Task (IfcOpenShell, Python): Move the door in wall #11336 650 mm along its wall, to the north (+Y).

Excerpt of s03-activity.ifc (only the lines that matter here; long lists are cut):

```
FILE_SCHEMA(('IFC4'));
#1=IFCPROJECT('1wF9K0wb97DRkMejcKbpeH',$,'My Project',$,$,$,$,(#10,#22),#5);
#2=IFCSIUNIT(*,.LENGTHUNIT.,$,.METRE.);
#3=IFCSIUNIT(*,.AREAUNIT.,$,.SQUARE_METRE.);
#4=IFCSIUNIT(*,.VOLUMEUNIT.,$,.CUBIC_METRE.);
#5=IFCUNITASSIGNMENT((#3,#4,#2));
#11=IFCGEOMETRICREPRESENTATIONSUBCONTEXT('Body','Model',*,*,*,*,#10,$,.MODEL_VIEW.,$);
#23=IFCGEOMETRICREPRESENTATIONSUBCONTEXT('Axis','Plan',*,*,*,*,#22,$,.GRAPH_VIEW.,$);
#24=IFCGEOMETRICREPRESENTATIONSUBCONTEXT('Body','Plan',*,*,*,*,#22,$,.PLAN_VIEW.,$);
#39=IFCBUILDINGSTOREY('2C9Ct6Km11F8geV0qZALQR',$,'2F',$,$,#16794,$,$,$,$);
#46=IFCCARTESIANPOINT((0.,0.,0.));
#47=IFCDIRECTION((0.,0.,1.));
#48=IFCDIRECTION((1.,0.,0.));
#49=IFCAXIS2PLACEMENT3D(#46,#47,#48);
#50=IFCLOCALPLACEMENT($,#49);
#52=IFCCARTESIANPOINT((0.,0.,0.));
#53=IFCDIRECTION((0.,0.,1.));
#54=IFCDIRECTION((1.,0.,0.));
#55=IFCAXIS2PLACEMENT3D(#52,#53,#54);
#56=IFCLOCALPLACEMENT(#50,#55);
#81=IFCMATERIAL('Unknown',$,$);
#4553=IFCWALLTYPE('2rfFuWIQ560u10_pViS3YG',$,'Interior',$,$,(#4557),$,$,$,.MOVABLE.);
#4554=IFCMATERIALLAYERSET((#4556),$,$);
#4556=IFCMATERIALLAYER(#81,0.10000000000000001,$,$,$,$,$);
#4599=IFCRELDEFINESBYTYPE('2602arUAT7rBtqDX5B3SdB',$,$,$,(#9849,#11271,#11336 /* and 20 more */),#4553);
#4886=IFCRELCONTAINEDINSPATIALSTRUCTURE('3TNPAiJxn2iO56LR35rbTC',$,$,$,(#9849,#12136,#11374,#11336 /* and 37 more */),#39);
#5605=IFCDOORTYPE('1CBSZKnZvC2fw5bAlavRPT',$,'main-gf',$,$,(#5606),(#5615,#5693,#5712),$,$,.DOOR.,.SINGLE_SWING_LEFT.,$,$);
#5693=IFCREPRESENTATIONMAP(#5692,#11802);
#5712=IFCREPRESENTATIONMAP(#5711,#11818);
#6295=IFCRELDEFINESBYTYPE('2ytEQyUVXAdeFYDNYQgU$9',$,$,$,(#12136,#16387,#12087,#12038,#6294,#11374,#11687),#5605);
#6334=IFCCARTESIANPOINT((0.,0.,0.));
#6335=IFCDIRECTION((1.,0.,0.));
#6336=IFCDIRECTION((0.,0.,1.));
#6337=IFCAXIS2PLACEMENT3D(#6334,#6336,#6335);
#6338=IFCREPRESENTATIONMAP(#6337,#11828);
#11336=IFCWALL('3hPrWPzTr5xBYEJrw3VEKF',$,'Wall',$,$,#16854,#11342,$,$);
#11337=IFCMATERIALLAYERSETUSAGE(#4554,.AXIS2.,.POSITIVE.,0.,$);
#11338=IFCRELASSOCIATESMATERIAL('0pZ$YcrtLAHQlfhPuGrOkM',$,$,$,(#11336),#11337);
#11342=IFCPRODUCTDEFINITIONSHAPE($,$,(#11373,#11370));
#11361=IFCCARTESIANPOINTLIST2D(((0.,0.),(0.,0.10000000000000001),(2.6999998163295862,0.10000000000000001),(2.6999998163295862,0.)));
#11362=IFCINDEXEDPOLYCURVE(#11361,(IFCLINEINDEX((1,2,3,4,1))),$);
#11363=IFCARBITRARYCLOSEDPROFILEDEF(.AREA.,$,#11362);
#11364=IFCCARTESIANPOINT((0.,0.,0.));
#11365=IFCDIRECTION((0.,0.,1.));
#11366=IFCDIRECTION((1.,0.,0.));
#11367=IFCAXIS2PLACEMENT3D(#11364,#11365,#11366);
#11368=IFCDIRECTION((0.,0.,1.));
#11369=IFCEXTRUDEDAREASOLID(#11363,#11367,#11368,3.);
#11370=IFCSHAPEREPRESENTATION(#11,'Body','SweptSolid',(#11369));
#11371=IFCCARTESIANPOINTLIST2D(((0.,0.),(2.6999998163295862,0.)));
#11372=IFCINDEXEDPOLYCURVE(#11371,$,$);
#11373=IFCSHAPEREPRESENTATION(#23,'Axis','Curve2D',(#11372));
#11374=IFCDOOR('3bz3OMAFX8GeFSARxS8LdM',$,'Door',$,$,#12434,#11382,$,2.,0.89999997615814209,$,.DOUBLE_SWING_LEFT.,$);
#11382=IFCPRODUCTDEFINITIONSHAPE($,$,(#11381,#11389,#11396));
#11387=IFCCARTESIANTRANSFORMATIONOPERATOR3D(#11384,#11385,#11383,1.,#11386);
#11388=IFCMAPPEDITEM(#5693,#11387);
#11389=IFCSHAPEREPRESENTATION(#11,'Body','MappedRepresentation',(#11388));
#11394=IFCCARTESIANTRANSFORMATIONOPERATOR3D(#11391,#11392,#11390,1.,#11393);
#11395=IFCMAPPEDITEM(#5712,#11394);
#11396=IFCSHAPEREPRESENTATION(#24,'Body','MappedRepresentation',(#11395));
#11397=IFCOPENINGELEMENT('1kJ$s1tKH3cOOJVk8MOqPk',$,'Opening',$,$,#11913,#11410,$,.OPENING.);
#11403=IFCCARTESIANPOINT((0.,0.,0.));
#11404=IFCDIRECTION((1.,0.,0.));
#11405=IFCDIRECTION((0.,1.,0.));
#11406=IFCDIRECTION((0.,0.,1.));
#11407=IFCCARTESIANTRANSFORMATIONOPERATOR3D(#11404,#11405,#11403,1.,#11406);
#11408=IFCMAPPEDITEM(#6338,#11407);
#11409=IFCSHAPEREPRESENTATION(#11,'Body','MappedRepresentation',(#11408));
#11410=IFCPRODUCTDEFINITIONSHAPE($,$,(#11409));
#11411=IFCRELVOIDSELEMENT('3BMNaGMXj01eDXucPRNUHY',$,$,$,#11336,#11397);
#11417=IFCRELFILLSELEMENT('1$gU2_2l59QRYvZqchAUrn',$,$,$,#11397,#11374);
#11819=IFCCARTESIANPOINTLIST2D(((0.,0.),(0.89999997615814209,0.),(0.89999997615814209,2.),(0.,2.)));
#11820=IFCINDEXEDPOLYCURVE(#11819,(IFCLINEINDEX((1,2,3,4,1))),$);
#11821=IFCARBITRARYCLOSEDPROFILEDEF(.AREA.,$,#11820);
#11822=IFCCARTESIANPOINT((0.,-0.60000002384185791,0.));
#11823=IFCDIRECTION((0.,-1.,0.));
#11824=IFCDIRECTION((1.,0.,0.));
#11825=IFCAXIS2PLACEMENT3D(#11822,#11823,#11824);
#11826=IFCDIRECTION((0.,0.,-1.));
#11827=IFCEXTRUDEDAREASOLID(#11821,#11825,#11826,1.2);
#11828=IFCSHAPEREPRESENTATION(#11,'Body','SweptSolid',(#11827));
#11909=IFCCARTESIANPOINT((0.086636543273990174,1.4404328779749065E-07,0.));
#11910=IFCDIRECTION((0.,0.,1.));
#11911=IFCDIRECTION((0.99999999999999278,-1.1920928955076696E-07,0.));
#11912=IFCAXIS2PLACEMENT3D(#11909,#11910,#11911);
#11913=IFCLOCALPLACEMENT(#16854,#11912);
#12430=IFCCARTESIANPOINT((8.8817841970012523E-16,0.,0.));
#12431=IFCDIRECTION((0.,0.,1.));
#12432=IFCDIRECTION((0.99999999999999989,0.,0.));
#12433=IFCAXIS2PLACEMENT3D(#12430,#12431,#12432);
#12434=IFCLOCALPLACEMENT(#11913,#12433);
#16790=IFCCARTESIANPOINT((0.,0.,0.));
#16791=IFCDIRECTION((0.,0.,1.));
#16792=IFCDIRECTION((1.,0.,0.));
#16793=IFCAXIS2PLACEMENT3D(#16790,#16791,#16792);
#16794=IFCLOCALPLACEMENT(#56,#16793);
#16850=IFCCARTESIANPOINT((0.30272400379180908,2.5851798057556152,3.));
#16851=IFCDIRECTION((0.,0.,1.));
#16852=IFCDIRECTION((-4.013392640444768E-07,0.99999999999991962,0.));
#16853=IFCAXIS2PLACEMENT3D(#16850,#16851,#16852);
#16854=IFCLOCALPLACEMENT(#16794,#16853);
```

```python
import ifcopenshell
import ifcopenshell.api.geometry
import ifcopenshell.util.placement
import ifcopenshell.util.unit

model = ifcopenshell.open("s03-activity.ifc")
unit_scale = ifcopenshell.util.unit.calculate_unit_scale(model)

door = model.by_id(11374)
opening = door.FillsVoids[0].RelatingOpeningElement
wall = opening.VoidsElements[0].RelatingBuildingElement

wall_matrix = ifcopenshell.util.placement.get_local_placement(wall.ObjectPlacement)
shift = wall_matrix[:3, 0] * 0.65 / unit_scale
before = ifcopenshell.util.placement.get_local_placement(door.ObjectPlacement)[:3, 3].copy()

# The door is placed relative to its opening, so it follows when the opening moves.
matrix = ifcopenshell.util.placement.get_local_placement(opening.ObjectPlacement)
matrix[:3, 3] += shift
ifcopenshell.api.geometry.edit_object_placement(
    model, product=opening, matrix=matrix, is_si=False, should_transform_children=True
)

after = ifcopenshell.util.placement.get_local_placement(door.ObjectPlacement)[:3, 3]
print("door moved by", (after - before).round(3) + 0.0)

model.write("s03-activity_v2.ifc")
```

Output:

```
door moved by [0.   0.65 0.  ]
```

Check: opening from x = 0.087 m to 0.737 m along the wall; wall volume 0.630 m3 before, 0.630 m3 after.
